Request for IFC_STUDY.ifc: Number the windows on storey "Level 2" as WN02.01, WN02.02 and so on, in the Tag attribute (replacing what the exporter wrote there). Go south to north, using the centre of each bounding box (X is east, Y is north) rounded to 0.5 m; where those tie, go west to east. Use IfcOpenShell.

First a look at what the model holds.

```python
import ifcopenshell
import ifcopenshell.util.element
import ifcopenshell.util.placement

model = ifcopenshell.open("IFC_STUDY.ifc")
print(model.schema)
storey = next(s for s in model.by_type("IfcBuildingStorey") if s.Name == "Level 2")
windows = [e for e in ifcopenshell.util.element.get_decomposition(storey) if e.is_a("IfcWindow")]
for e in sorted(windows, key=lambda e: e.id()):
    origin = ifcopenshell.util.placement.get_local_placement(e.ObjectPlacement)[:3, 3]
    print(e.id(), e.Tag, e.Name, origin.round(2) + 0.0, sep=" | ")
```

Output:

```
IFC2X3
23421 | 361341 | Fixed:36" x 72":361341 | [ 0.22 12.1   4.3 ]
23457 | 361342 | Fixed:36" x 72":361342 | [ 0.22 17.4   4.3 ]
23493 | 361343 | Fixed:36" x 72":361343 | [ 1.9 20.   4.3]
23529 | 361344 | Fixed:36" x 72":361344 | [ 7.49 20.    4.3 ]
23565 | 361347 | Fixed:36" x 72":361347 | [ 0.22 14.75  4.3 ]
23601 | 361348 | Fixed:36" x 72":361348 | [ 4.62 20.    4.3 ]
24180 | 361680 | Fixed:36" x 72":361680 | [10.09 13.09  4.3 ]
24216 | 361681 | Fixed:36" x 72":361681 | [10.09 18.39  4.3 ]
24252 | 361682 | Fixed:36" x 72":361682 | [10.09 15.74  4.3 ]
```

```python
import ifcopenshell
import ifcopenshell.geom
import ifcopenshell.util.element
import ifcopenshell.util.shape

model = ifcopenshell.open("IFC_STUDY.ifc")
settings = ifcopenshell.geom.settings()
settings.set("use-world-coords", True)


def centre(element):
    shape = ifcopenshell.geom.create_shape(settings, element)
    return ifcopenshell.util.shape.get_bbox_centroid(shape.geometry)


storey = next(s for s in model.by_type("IfcBuildingStorey") if s.Name == "Level 2")
windows = [e for e in ifcopenshell.util.element.get_decomposition(storey) if e.is_a("IfcWindow")]

# Insertion points can sit at a corner or the storey origin, so sort by the geometry (in metres).
centres = {e: centre(e) for e in windows}
windows.sort(key=lambda e: (round(centres[e][1] / 0.5), centres[e][0]))

for i, e in enumerate(windows, start=1):
    number = f"WN02.{i:02d}"
    e.Tag = number
    print(e.id(), number)

model.write("IFC_STUDY_edited.ifc")
```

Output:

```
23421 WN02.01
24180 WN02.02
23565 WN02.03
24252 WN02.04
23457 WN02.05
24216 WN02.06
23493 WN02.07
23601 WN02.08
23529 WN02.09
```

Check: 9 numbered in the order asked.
